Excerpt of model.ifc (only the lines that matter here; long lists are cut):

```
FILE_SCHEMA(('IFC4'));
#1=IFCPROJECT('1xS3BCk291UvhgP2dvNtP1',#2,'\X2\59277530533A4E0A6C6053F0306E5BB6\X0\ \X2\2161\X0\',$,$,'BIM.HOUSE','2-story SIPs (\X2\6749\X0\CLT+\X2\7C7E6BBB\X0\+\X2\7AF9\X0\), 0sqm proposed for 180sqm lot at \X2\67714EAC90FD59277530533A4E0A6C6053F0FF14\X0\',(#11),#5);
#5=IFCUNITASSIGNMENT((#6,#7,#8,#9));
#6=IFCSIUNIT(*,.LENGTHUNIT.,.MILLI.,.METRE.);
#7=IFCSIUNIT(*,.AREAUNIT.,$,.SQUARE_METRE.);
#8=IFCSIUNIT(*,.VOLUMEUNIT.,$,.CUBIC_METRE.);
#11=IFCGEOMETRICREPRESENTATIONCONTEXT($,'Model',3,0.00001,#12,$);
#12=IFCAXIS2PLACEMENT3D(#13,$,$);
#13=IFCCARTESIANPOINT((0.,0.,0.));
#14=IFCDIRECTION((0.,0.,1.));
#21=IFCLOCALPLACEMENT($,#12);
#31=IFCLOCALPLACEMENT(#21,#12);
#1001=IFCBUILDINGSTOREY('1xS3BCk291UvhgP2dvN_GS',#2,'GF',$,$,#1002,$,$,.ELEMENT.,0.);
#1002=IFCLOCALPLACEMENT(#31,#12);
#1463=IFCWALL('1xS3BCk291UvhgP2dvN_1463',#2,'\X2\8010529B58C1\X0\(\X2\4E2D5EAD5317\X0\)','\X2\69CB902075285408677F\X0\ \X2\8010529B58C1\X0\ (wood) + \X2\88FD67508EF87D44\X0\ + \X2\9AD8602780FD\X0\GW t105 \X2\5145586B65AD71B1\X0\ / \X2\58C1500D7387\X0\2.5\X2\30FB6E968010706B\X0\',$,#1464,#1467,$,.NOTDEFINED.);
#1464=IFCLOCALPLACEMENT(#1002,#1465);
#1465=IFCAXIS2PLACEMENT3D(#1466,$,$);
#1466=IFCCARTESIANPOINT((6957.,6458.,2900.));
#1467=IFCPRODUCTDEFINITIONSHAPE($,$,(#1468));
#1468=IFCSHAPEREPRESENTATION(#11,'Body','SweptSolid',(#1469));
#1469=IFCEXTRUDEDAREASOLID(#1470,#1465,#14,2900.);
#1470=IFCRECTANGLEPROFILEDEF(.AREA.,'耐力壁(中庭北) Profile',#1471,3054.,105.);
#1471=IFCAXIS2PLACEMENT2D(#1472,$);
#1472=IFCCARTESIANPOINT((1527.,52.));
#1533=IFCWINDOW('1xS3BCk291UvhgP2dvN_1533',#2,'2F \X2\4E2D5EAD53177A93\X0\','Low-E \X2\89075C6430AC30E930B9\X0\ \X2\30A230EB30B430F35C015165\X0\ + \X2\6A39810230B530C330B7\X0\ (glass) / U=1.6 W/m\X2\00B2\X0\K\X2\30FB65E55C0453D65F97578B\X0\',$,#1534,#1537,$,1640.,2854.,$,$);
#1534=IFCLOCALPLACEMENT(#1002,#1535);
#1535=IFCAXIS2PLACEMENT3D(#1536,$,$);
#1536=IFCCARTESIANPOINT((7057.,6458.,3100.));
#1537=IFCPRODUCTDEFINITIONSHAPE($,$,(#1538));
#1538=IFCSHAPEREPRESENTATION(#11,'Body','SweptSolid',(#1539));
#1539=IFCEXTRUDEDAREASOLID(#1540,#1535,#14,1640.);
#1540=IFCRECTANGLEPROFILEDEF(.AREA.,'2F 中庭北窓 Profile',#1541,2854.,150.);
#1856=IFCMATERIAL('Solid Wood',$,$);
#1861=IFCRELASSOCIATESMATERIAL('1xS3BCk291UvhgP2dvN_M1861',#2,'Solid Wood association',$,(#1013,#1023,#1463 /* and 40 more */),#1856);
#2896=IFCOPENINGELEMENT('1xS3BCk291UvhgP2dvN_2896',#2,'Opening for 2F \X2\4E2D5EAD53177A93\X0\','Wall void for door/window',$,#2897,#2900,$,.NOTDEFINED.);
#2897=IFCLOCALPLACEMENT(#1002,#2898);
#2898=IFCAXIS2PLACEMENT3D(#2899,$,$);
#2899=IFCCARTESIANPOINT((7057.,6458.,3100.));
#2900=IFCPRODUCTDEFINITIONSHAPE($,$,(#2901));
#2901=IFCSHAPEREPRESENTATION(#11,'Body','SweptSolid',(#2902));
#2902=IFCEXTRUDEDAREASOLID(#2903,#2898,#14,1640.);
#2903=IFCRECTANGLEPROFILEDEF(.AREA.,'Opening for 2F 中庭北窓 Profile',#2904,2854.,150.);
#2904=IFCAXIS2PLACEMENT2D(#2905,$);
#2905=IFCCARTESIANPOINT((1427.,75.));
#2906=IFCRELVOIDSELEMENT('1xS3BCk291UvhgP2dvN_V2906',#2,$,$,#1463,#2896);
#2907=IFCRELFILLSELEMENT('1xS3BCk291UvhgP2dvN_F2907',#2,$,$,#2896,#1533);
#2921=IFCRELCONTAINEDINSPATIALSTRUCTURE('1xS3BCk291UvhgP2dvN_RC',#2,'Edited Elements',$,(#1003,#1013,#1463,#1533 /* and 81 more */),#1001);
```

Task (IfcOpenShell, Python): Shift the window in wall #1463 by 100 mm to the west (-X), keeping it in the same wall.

```python
import ifcopenshell
import ifcopenshell.api.geometry
import ifcopenshell.util.placement
import ifcopenshell.util.unit

model = ifcopenshell.open("model.ifc")
unit_scale = ifcopenshell.util.unit.calculate_unit_scale(model)

window = model.by_guid("1xS3BCk291UvhgP2dvN_1533")
opening = window.FillsVoids[0].RelatingOpeningElement
wall = opening.VoidsElements[0].RelatingBuildingElement

wall_matrix = ifcopenshell.util.placement.get_local_placement(wall.ObjectPlacement)
shift = wall_matrix[:3, 0] * -0.1 / unit_scale
before = ifcopenshell.util.placement.get_local_placement(window.ObjectPlacement)[:3, 3].copy()

# The window is not placed relative to its opening, so move both.
for product in (opening, window):
    matrix = ifcopenshell.util.placement.get_local_placement(product.ObjectPlacement)
    matrix[:3, 3] += shift
    ifcopenshell.api.geometry.edit_object_placement(model, product=product, matrix=matrix, is_si=False)

after = ifcopenshell.util.placement.get_local_placement(window.ObjectPlacement)[:3, 3]
print("window moved by", (after - before).round(3) + 0.0)

model.write("model_edited.ifc")
```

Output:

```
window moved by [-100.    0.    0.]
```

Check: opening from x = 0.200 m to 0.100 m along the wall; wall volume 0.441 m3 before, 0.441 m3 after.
